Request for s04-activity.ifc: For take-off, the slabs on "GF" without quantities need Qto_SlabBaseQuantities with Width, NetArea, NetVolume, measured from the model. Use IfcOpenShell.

First a look at what the model holds.

```python
import ifcopenshell
import ifcopenshell.util.element
import ifcopenshell.util.unit

model = ifcopenshell.open("s04-activity.ifc")
print(model.schema)
for unit_type in ("LENGTHUNIT", "AREAUNIT", "VOLUMEUNIT"):
    print(unit_type, ifcopenshell.util.unit.calculate_unit_scale(model, unit_type))
storey = next(s for s in model.by_type("IfcBuildingStorey") if s.Name == "GF")
slabs = [e for e in ifcopenshell.util.element.get_decomposition(storey) if e.is_a("IfcSlab")]
for e in sorted(slabs, key=lambda e: e.id()):
    print(e.id(), e.is_a(), e.Name, list(ifcopenshell.util.element.get_psets(e, qtos_only=True)), sep=" | ")
```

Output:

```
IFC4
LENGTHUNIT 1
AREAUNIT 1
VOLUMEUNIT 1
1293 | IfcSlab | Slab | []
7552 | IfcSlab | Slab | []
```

```python
import ifcopenshell
import ifcopenshell.api.pset
import ifcopenshell.geom
import ifcopenshell.util.element
import ifcopenshell.util.shape
import ifcopenshell.util.unit

model = ifcopenshell.open("s04-activity.ifc")
unit_scale = ifcopenshell.util.unit.calculate_unit_scale(model)
area_scale = ifcopenshell.util.unit.calculate_unit_scale(model, "AREAUNIT")
volume_scale = ifcopenshell.util.unit.calculate_unit_scale(model, "VOLUMEUNIT")
settings = ifcopenshell.geom.settings()

storey = next(s for s in model.by_type("IfcBuildingStorey") if s.Name == "GF")
slabs = [e for e in ifcopenshell.util.element.get_decomposition(storey) if e.is_a("IfcSlab")]

for e in sorted(slabs, key=lambda e: e.id()):
    if ifcopenshell.util.element.get_psets(e, qtos_only=True, should_inherit=False):
        continue
    # Geometry comes back in metres, in the element's own axes.
    shape = ifcopenshell.geom.create_shape(settings, e)
    values = {
        "Width": ifcopenshell.util.shape.get_z(shape.geometry) / unit_scale,
        "NetArea": ifcopenshell.util.shape.get_footprint_area(shape.geometry) / area_scale,
        "NetVolume": ifcopenshell.util.shape.get_volume(shape.geometry) / volume_scale,
    }
    qto = ifcopenshell.api.pset.add_qto(model, product=e, name="Qto_SlabBaseQuantities")
    ifcopenshell.api.pset.edit_qto(model, qto=qto, properties=values)
    print(e.id(), {k: round(v, 3) for k, v in values.items()})

model.write("s04-activity_rev.ifc")
```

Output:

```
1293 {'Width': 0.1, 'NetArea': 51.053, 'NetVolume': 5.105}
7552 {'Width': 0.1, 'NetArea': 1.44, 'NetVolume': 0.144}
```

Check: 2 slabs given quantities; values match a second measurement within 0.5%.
